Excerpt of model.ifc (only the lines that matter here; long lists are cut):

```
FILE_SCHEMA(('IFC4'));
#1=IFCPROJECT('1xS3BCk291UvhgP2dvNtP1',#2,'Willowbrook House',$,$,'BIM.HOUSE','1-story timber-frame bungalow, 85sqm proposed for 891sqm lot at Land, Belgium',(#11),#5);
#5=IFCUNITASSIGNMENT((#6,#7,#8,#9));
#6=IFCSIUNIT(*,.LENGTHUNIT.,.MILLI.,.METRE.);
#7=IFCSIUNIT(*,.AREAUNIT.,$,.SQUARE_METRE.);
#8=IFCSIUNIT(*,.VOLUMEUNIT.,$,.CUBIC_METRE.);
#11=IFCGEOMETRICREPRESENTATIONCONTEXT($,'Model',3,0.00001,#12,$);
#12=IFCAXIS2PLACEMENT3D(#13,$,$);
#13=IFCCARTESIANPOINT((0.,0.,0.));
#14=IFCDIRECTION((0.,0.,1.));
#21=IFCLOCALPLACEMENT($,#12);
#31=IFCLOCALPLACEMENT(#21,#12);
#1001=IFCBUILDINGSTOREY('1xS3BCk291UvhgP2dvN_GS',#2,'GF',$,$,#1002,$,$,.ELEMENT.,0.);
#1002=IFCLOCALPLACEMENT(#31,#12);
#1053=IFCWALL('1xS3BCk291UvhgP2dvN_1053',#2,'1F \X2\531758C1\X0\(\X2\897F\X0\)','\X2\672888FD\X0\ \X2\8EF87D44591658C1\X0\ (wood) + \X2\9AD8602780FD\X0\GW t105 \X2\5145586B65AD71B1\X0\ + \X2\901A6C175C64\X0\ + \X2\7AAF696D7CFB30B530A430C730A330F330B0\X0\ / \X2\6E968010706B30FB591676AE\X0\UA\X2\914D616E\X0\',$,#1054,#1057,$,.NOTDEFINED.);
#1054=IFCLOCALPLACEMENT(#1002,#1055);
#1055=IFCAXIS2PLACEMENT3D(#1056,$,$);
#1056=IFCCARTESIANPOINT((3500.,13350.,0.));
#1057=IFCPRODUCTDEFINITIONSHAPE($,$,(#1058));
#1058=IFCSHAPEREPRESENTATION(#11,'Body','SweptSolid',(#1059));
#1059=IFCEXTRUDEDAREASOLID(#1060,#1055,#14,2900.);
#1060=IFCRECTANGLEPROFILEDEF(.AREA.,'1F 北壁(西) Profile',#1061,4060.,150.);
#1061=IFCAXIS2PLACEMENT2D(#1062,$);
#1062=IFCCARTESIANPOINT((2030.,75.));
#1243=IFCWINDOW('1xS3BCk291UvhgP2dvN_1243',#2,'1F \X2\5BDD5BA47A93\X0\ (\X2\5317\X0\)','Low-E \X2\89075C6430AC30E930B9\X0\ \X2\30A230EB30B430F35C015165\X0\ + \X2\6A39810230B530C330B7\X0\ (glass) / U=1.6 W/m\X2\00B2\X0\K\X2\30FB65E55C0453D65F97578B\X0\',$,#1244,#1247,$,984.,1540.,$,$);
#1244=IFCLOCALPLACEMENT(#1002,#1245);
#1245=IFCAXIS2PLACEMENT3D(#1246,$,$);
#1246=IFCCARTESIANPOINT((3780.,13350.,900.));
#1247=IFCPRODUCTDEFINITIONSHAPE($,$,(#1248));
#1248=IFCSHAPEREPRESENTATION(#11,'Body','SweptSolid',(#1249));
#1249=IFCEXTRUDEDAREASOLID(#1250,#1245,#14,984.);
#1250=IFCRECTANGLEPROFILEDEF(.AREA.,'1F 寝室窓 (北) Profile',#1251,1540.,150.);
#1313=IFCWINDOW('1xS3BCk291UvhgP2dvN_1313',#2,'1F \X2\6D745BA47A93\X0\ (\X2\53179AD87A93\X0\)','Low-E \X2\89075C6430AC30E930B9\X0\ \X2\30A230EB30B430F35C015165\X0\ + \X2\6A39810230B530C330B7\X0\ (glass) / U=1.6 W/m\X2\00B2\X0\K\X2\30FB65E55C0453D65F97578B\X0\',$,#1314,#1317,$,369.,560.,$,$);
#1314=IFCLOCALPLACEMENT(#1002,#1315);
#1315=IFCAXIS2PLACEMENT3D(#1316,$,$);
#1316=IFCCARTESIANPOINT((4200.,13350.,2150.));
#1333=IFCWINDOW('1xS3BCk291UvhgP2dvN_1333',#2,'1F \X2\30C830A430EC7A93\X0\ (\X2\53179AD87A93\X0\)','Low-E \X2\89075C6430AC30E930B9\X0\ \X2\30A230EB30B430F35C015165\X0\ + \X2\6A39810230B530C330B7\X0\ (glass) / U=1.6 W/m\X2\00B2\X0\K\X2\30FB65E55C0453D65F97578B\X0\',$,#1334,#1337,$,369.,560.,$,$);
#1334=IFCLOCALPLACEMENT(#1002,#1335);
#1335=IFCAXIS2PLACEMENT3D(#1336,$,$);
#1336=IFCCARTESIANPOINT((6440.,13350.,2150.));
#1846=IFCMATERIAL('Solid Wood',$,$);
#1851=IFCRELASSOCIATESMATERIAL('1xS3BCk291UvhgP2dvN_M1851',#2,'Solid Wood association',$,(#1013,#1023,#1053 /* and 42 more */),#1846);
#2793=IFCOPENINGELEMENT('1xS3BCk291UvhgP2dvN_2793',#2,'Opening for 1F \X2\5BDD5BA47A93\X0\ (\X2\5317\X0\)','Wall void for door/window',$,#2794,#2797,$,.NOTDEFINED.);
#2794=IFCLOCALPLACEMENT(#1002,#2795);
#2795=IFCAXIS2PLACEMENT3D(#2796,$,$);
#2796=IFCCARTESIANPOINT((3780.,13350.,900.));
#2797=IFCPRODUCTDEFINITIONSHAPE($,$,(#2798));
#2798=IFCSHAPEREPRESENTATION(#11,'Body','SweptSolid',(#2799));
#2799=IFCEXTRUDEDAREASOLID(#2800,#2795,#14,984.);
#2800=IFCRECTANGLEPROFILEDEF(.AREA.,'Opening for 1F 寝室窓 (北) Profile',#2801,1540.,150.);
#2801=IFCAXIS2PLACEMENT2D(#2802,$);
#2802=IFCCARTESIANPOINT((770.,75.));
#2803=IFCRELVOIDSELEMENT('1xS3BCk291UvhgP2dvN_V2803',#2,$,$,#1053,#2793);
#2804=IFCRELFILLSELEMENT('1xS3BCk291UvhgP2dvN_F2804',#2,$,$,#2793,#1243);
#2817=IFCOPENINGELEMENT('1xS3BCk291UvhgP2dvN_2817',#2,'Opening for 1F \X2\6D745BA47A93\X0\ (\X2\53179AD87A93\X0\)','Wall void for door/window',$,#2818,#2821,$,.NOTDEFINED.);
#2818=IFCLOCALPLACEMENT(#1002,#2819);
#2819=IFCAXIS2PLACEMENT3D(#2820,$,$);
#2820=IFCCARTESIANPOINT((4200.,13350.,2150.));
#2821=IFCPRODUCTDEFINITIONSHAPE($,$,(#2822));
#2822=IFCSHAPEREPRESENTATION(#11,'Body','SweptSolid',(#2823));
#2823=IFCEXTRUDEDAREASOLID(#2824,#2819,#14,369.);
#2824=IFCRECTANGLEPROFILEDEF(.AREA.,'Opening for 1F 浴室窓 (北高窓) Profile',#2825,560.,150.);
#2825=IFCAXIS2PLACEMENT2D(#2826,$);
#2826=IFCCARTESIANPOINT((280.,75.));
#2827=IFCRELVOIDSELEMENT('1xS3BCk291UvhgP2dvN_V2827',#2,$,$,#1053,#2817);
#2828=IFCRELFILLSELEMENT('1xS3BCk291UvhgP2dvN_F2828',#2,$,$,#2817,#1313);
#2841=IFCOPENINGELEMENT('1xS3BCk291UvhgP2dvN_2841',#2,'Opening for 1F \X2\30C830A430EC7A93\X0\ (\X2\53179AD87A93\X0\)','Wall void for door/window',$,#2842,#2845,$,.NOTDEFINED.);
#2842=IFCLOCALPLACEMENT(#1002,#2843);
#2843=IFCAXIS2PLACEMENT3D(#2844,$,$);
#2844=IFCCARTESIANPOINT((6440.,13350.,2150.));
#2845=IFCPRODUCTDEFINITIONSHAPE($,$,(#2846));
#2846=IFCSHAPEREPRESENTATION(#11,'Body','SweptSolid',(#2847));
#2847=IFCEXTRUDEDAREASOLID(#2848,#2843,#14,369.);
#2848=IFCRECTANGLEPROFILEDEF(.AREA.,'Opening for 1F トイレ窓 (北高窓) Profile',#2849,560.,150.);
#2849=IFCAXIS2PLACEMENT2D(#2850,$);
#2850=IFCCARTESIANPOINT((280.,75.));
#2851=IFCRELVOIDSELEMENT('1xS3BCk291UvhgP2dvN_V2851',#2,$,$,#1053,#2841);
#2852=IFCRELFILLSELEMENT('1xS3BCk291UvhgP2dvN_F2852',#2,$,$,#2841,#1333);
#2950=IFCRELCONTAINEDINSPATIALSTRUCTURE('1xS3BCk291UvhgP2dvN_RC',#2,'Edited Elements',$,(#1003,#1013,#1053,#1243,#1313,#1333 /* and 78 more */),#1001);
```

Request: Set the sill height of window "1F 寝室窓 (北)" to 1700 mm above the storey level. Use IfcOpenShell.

```python
import numpy as np
import ifcopenshell
import ifcopenshell.api.geometry
import ifcopenshell.geom
import ifcopenshell.util.element
import ifcopenshell.util.placement
import ifcopenshell.util.shape
import ifcopenshell.util.unit

model = ifcopenshell.open("model.ifc")
unit_scale = ifcopenshell.util.unit.calculate_unit_scale(model)

window = model.by_guid("1xS3BCk291UvhgP2dvN_1243")
opening = window.FillsVoids[0].RelatingOpeningElement
storey = ifcopenshell.util.element.get_container(window, ifc_class="IfcBuildingStorey")
level = ifcopenshell.util.placement.get_local_placement(storey.ObjectPlacement)[2, 3]

# The opening's origin need not be at the sill, so measure its lowest point.
shape = ifcopenshell.geom.create_shape(ifcopenshell.geom.settings(), opening)
bottom = ifcopenshell.util.shape.get_shape_bottom_elevation(shape, shape.geometry) / unit_scale
dz = level + 1700.0 - bottom

shift = np.array([0.0, 0.0, dz])
# The window is not placed relative to its opening, so move both.
for product in (opening, window):
    matrix = ifcopenshell.util.placement.get_local_placement(product.ObjectPlacement)
    matrix[:3, 3] += shift
    ifcopenshell.api.geometry.edit_object_placement(model, product=product, matrix=matrix, is_si=False)

print(f"moved by {dz * unit_scale:+.3f} m")

model.write("model_v2.ifc")
```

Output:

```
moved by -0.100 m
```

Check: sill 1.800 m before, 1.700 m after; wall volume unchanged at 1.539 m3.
